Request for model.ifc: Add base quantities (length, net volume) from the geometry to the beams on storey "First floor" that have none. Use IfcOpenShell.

First a look at what the model holds.

```python
import ifcopenshell
import ifcopenshell.util.element
import ifcopenshell.util.unit

model = ifcopenshell.open("model.ifc")
print(model.schema)
for unit_type in ("LENGTHUNIT", "AREAUNIT", "VOLUMEUNIT"):
    print(unit_type, ifcopenshell.util.unit.calculate_unit_scale(model, unit_type))
storey = next(s for s in model.by_type("IfcBuildingStorey") if s.Name == "First floor")
beams = [e for e in ifcopenshell.util.element.get_decomposition(storey) if e.is_a("IfcBeam")]
for e in sorted(beams, key=lambda e: e.id()):
    print(e.id(), e.is_a(), e.Name, list(ifcopenshell.util.element.get_psets(e, qtos_only=True)), sep=" | ")
```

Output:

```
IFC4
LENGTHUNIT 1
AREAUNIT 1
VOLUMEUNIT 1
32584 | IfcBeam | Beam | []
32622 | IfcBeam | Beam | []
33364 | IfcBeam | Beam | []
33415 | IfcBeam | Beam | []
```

```python
import ifcopenshell
import ifcopenshell.api.pset
import ifcopenshell.geom
import ifcopenshell.util.element
import ifcopenshell.util.shape
import ifcopenshell.util.unit

model = ifcopenshell.open("model.ifc")
unit_scale = ifcopenshell.util.unit.calculate_unit_scale(model)
volume_scale = ifcopenshell.util.unit.calculate_unit_scale(model, "VOLUMEUNIT")
settings = ifcopenshell.geom.settings()

storey = next(s for s in model.by_type("IfcBuildingStorey") if s.Name == "First floor")
beams = [e for e in ifcopenshell.util.element.get_decomposition(storey) if e.is_a("IfcBeam")]

for e in sorted(beams, key=lambda e: e.id()):
    if ifcopenshell.util.element.get_psets(e, qtos_only=True, should_inherit=False):
        continue
    # Geometry comes back in metres, in the element's own axes.
    shape = ifcopenshell.geom.create_shape(settings, e)
    values = {
        "Length": ifcopenshell.util.shape.get_max_xyz(shape.geometry) / unit_scale,
        "NetVolume": ifcopenshell.util.shape.get_volume(shape.geometry) / volume_scale,
    }
    qto = ifcopenshell.api.pset.add_qto(model, product=e, name="Qto_BeamBaseQuantities")
    ifcopenshell.api.pset.edit_qto(model, qto=qto, properties=values)
    print(e.id(), {k: round(v, 3) for k, v in values.items()})

model.write("model-out.ifc")
```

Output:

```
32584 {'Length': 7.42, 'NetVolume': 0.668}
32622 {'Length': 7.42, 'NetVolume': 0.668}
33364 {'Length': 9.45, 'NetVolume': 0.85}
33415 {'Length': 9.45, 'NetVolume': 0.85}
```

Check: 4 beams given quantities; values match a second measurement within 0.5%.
